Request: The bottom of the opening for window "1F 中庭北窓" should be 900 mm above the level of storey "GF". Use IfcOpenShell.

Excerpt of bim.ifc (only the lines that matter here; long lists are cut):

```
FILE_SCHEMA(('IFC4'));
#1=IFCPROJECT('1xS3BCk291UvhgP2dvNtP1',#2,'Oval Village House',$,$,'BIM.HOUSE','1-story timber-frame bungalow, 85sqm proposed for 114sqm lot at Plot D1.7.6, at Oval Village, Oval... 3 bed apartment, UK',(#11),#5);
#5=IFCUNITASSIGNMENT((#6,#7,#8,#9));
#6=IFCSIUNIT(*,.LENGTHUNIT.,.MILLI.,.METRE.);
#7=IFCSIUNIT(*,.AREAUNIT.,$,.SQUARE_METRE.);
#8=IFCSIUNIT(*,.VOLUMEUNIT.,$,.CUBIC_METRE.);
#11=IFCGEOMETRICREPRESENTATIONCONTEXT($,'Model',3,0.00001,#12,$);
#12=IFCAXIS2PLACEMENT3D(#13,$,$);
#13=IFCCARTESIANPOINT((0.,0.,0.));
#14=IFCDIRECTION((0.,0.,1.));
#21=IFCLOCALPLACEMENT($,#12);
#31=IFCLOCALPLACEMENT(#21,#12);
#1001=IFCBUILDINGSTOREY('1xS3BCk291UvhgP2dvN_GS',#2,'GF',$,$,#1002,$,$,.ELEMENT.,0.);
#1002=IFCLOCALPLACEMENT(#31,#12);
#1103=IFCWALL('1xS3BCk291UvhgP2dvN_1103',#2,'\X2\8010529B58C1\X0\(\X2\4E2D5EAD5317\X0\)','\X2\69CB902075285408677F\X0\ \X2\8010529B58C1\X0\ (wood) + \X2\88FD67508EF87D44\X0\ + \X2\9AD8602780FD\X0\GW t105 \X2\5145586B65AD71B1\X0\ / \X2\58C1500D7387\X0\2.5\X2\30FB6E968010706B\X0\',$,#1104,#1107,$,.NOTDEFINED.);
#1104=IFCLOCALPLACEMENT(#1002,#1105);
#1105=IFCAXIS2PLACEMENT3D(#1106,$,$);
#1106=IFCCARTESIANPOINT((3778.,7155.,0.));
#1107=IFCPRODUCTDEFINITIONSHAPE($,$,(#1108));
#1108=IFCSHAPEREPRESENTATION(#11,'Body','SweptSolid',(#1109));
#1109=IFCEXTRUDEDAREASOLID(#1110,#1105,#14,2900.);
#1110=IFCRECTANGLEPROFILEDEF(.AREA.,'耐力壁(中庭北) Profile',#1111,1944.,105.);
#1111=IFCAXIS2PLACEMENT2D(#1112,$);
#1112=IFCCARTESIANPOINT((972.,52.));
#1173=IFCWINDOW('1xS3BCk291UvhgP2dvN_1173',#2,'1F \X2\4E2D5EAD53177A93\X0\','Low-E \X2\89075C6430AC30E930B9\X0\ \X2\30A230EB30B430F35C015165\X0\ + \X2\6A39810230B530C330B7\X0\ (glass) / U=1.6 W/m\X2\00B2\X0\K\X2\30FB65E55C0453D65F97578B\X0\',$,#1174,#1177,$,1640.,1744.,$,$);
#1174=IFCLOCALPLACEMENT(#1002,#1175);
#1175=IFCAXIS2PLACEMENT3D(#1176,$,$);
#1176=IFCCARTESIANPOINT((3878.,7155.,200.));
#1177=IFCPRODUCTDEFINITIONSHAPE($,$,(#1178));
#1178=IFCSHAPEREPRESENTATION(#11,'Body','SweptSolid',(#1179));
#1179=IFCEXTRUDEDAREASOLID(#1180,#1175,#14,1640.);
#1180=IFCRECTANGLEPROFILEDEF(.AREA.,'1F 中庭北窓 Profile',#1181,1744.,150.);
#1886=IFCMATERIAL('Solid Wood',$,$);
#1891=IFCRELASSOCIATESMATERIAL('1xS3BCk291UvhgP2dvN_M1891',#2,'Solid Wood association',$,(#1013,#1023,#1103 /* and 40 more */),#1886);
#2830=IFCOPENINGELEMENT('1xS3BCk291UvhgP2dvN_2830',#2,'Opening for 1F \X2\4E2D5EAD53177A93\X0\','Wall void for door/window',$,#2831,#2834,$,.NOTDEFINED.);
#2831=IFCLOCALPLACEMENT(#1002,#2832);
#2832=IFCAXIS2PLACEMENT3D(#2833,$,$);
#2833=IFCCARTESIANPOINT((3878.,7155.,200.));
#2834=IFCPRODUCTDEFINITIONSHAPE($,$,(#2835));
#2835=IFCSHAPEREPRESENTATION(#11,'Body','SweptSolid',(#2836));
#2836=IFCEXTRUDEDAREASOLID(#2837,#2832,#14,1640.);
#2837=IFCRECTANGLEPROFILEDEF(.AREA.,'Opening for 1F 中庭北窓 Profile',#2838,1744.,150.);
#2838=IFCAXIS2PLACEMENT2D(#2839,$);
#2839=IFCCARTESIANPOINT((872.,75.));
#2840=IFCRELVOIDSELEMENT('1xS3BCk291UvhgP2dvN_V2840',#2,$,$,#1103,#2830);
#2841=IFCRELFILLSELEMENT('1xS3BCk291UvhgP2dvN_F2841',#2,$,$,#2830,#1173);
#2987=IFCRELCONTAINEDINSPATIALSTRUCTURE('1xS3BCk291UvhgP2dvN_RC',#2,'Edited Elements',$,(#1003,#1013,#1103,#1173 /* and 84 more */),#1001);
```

```python
import numpy as np
import ifcopenshell
import ifcopenshell.api.geometry
import ifcopenshell.geom
import ifcopenshell.util.element
import ifcopenshell.util.placement
import ifcopenshell.util.shape
import ifcopenshell.util.unit

model = ifcopenshell.open("bim.ifc")
unit_scale = ifcopenshell.util.unit.calculate_unit_scale(model)

window = model.by_guid("1xS3BCk291UvhgP2dvN_1173")
opening = window.FillsVoids[0].RelatingOpeningElement
storey = ifcopenshell.util.element.get_container(window, ifc_class="IfcBuildingStorey")
level = ifcopenshell.util.placement.get_local_placement(storey.ObjectPlacement)[2, 3]

# The opening's origin need not be at the sill, so measure its lowest point.
shape = ifcopenshell.geom.create_shape(ifcopenshell.geom.settings(), opening)
bottom = ifcopenshell.util.shape.get_shape_bottom_elevation(shape, shape.geometry) / unit_scale
dz = level + 0.9 / unit_scale - bottom

shift = np.array([0.0, 0.0, dz])
# The window is not placed relative to its opening, so move both.
for product in (opening, window):
    matrix = ifcopenshell.util.placement.get_local_placement(product.ObjectPlacement)
    matrix[:3, 3] += shift
    ifcopenshell.api.geometry.edit_object_placement(model, product=product, matrix=matrix, is_si=False)

print(f"moved by {dz * unit_scale:+.3f} m")

model.write("bim_v2.ifc")
```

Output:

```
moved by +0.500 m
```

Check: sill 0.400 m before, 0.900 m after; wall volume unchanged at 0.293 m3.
